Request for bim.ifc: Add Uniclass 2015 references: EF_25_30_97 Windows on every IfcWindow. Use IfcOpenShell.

First a look at what the model holds.

```python
import ifcopenshell

model = ifcopenshell.open("bim.ifc")
print(model.schema)
print("classifications:", [c.Name for c in model.by_type("IfcClassification")])
for ifc_class in ("IfcDoor", "IfcRoof", "IfcStair", "IfcWall", "IfcWindow"):
    print(ifc_class, len(model.by_type(ifc_class)))
```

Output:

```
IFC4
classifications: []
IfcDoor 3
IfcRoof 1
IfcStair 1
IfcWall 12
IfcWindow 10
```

```python
import ifcopenshell
import ifcopenshell.api.classification

model = ifcopenshell.open("bim.ifc")

system = ifcopenshell.api.classification.add_classification(model, classification="Uniclass 2015")

codes = {
    "IfcWindow": ("EF_25_30_97", "Windows"),
}
for ifc_class, (code, name) in codes.items():
    products = model.by_type(ifc_class)
    ifcopenshell.api.classification.add_reference(
        model, products=products, classification=system, identification=code, name=name
    )
    print(code, len(products))

model.write("bim-out.ifc")
```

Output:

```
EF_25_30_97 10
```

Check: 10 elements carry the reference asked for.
